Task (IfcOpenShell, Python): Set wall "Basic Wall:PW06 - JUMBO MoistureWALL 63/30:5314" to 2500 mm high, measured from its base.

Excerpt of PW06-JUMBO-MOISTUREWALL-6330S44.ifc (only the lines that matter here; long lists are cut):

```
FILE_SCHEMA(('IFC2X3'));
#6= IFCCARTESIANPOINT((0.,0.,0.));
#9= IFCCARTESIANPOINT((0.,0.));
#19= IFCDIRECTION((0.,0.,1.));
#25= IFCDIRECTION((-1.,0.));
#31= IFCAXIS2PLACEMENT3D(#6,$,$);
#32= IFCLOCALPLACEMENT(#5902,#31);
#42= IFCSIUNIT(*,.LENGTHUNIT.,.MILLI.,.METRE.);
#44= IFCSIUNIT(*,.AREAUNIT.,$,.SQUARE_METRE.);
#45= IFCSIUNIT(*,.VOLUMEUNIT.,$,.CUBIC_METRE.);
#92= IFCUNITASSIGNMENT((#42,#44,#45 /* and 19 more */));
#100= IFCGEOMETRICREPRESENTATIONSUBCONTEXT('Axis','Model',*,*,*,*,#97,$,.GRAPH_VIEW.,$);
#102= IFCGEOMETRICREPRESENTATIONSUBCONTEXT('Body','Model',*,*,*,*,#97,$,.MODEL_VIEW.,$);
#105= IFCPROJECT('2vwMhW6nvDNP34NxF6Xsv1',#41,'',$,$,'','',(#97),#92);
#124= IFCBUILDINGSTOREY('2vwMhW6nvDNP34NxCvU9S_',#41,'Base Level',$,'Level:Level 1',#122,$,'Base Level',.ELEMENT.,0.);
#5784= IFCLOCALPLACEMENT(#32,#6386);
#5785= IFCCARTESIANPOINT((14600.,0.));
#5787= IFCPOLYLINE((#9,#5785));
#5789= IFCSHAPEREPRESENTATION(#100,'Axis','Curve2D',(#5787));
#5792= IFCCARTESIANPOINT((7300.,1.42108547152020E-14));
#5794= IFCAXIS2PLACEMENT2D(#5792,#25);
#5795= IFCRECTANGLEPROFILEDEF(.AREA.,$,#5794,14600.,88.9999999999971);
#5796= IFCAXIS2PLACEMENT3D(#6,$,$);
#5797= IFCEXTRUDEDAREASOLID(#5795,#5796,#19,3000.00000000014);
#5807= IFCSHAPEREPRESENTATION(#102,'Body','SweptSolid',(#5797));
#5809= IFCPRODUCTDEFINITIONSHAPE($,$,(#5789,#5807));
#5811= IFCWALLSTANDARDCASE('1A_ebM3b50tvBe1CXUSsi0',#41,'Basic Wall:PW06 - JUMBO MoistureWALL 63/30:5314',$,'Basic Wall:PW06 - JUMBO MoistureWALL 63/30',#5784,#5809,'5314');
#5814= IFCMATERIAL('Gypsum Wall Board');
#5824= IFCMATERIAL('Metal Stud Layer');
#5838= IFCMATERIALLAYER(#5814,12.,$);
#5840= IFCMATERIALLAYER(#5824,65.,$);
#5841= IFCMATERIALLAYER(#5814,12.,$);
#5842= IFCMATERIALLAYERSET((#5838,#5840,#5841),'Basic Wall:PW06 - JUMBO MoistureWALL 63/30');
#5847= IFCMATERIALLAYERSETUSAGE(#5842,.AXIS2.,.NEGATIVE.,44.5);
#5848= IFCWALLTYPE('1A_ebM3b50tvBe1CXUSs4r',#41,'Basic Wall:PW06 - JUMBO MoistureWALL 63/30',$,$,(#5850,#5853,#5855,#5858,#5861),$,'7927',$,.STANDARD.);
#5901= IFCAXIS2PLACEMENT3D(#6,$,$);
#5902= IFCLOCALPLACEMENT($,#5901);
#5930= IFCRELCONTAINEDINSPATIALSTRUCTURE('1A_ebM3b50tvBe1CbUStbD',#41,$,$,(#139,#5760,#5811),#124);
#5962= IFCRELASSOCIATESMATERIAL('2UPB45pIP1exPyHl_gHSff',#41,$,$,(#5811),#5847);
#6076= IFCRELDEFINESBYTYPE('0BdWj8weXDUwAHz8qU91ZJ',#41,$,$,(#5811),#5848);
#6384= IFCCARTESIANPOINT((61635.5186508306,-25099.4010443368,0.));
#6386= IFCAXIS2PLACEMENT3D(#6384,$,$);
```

```python
import ifcopenshell
import ifcopenshell.geom
import ifcopenshell.util.representation
import ifcopenshell.util.shape
import ifcopenshell.util.unit

model = ifcopenshell.open("PW06-JUMBO-MOISTUREWALL-6330S44.ifc")
unit_scale = ifcopenshell.util.unit.calculate_unit_scale(model)
settings = ifcopenshell.geom.settings()


def volume(element):
    """Net volume in cubic metres, openings subtracted."""
    shape = ifcopenshell.geom.create_shape(settings, element)
    return ifcopenshell.util.shape.get_volume(shape.geometry)


wall = model.by_id(5811)
before = volume(wall)

body = ifcopenshell.util.representation.get_representation(wall, "Model", "Body")
solid = body.Items[0]
old_height = solid.Depth
solid.Depth = 2.5 / unit_scale
after = volume(wall)

print(f"height {old_height:g} -> {solid.Depth:g}, volume {before:.3f} -> {after:.3f} m3")

model.write("PW06-JUMBO-MOISTUREWALL-6330S44_v2.ifc")
```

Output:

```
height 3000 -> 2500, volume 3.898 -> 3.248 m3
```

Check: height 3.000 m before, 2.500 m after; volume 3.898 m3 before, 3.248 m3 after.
